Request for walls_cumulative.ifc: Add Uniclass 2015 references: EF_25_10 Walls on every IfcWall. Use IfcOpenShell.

First a look at what the model holds.

```python
import ifcopenshell

model = ifcopenshell.open("walls_cumulative.ifc")
print(model.schema)
print("classifications:", [c.Name for c in model.by_type("IfcClassification")])
for ifc_class in ("IfcDoor", "IfcRoof", "IfcStair", "IfcWall", "IfcWindow"):
    print(ifc_class, len(model.by_type(ifc_class)))
```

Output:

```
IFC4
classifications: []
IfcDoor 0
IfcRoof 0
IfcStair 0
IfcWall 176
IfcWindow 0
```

```python
import ifcopenshell
import ifcopenshell.api.classification

model = ifcopenshell.open("walls_cumulative.ifc")

system = ifcopenshell.api.classification.add_classification(model, classification="Uniclass 2015")

codes = {
    "IfcWall": ("EF_25_10", "Walls"),
}
for ifc_class, (code, name) in codes.items():
    products = model.by_type(ifc_class)
    ifcopenshell.api.classification.add_reference(
        model, products=products, classification=system, identification=code, name=name
    )
    print(code, len(products))

model.write("walls_cumulative_rev.ifc")
```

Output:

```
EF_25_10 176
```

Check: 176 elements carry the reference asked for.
